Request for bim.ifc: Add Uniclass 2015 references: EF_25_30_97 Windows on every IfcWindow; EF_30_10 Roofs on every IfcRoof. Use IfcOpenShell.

First a look at what the model holds.

```python
import ifcopenshell

model = ifcopenshell.open("bim.ifc")
print(model.schema)
print("classifications:", [c.Name for c in model.by_type("IfcClassification")])
for ifc_class in ("IfcDoor", "IfcRoof", "IfcStair", "IfcWall", "IfcWindow"):
    print(ifc_class, len(model.by_type(ifc_class)))
```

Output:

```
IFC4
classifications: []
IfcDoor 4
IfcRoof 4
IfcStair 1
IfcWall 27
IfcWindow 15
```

```python
import ifcopenshell
import ifcopenshell.api.classification

model = ifcopenshell.open("bim.ifc")

system = ifcopenshell.api.classification.add_classification(model, classification="Uniclass 2015")

codes = {
    "IfcWindow": ("EF_25_30_97", "Windows"),
    "IfcRoof": ("EF_30_10", "Roofs"),
}
for ifc_class, (code, name) in codes.items():
    products = model.by_type(ifc_class)
    ifcopenshell.api.classification.add_reference(
        model, products=products, classification=system, identification=code, name=name
    )
    print(code, len(products))

model.write("bim_edited.ifc")
```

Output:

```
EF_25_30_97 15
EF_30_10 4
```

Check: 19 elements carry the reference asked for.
